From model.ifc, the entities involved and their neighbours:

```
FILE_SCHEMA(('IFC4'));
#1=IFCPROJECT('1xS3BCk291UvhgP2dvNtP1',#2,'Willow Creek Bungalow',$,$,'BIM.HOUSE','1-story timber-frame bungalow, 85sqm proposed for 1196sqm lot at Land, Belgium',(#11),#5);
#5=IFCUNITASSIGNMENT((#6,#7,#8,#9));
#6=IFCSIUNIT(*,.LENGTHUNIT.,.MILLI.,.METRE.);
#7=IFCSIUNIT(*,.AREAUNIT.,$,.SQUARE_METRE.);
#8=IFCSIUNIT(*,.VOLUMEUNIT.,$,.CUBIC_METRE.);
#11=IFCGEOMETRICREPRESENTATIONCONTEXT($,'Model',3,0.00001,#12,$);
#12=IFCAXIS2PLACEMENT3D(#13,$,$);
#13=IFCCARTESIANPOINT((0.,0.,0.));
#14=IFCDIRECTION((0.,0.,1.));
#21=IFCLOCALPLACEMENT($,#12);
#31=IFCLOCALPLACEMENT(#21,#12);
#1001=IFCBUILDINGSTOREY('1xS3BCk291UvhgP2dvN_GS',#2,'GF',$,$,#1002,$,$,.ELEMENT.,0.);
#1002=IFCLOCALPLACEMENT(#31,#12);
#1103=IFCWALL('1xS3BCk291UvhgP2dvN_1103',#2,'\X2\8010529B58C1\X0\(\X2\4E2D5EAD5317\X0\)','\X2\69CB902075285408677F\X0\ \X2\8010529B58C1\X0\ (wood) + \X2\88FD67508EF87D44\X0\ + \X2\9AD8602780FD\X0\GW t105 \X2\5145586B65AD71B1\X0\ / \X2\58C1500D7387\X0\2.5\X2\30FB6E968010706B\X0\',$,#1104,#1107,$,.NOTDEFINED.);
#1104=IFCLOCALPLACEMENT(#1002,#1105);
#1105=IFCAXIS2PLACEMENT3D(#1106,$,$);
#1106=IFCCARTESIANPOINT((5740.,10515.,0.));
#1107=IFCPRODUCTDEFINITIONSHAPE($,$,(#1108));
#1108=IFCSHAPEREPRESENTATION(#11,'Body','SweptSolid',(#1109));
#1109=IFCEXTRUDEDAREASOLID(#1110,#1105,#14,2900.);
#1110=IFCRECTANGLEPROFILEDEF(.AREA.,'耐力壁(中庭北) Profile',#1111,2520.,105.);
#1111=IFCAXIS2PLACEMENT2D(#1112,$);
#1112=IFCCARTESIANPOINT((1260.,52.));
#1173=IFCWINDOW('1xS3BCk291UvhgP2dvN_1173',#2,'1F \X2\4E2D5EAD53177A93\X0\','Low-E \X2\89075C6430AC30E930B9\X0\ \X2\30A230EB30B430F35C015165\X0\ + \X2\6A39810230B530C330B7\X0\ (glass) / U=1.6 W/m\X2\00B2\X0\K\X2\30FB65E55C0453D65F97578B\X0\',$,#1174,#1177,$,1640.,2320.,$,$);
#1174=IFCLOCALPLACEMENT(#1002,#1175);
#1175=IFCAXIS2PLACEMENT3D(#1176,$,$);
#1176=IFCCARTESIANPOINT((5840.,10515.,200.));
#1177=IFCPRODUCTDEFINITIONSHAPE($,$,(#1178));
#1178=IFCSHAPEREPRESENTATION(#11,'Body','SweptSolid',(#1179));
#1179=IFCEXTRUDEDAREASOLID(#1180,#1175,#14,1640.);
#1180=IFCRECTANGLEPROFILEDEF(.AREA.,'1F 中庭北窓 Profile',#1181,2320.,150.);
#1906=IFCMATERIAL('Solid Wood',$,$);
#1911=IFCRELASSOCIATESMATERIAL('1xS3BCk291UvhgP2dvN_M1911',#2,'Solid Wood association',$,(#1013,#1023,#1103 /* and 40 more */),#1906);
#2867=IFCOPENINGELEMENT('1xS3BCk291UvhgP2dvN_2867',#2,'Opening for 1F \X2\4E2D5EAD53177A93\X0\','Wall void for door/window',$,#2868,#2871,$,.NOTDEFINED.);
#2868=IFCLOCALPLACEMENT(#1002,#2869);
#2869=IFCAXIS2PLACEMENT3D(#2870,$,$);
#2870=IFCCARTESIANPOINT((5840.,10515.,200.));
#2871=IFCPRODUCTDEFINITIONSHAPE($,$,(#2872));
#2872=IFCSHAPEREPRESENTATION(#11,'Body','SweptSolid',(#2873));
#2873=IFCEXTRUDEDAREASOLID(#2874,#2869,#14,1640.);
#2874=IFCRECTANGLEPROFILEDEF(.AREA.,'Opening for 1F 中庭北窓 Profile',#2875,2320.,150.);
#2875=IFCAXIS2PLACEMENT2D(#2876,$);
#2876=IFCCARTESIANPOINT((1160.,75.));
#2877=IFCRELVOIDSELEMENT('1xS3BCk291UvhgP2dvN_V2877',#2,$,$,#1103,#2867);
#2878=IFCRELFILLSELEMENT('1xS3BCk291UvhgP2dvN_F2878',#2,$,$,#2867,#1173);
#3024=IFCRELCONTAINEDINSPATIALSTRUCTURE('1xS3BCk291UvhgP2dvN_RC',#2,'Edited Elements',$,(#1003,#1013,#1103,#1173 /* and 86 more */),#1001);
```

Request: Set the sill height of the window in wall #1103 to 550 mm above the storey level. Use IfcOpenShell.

```python
import numpy as np
import ifcopenshell
import ifcopenshell.api.geometry
import ifcopenshell.geom
import ifcopenshell.util.element
import ifcopenshell.util.placement
import ifcopenshell.util.shape
import ifcopenshell.util.unit

model = ifcopenshell.open("model.ifc")
unit_scale = ifcopenshell.util.unit.calculate_unit_scale(model)

window = model.by_id(1173)
opening = window.FillsVoids[0].RelatingOpeningElement
storey = ifcopenshell.util.element.get_container(window, ifc_class="IfcBuildingStorey")
level = ifcopenshell.util.placement.get_local_placement(storey.ObjectPlacement)[2, 3]

# The opening's origin need not be at the sill, so measure its lowest point.
shape = ifcopenshell.geom.create_shape(ifcopenshell.geom.settings(), opening)
bottom = ifcopenshell.util.shape.get_shape_bottom_elevation(shape, shape.geometry) / unit_scale
dz = level + 550.0 - bottom

shift = np.array([0.0, 0.0, dz])
# The window is not placed relative to its opening, so move both.
for product in (opening, window):
    matrix = ifcopenshell.util.placement.get_local_placement(product.ObjectPlacement)
    matrix[:3, 3] += shift
    ifcopenshell.api.geometry.edit_object_placement(model, product=product, matrix=matrix, is_si=False)

print(f"moved by {dz * unit_scale:+.3f} m")

model.write("model-out.ifc")
```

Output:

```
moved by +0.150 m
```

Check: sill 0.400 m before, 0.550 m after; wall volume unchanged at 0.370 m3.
